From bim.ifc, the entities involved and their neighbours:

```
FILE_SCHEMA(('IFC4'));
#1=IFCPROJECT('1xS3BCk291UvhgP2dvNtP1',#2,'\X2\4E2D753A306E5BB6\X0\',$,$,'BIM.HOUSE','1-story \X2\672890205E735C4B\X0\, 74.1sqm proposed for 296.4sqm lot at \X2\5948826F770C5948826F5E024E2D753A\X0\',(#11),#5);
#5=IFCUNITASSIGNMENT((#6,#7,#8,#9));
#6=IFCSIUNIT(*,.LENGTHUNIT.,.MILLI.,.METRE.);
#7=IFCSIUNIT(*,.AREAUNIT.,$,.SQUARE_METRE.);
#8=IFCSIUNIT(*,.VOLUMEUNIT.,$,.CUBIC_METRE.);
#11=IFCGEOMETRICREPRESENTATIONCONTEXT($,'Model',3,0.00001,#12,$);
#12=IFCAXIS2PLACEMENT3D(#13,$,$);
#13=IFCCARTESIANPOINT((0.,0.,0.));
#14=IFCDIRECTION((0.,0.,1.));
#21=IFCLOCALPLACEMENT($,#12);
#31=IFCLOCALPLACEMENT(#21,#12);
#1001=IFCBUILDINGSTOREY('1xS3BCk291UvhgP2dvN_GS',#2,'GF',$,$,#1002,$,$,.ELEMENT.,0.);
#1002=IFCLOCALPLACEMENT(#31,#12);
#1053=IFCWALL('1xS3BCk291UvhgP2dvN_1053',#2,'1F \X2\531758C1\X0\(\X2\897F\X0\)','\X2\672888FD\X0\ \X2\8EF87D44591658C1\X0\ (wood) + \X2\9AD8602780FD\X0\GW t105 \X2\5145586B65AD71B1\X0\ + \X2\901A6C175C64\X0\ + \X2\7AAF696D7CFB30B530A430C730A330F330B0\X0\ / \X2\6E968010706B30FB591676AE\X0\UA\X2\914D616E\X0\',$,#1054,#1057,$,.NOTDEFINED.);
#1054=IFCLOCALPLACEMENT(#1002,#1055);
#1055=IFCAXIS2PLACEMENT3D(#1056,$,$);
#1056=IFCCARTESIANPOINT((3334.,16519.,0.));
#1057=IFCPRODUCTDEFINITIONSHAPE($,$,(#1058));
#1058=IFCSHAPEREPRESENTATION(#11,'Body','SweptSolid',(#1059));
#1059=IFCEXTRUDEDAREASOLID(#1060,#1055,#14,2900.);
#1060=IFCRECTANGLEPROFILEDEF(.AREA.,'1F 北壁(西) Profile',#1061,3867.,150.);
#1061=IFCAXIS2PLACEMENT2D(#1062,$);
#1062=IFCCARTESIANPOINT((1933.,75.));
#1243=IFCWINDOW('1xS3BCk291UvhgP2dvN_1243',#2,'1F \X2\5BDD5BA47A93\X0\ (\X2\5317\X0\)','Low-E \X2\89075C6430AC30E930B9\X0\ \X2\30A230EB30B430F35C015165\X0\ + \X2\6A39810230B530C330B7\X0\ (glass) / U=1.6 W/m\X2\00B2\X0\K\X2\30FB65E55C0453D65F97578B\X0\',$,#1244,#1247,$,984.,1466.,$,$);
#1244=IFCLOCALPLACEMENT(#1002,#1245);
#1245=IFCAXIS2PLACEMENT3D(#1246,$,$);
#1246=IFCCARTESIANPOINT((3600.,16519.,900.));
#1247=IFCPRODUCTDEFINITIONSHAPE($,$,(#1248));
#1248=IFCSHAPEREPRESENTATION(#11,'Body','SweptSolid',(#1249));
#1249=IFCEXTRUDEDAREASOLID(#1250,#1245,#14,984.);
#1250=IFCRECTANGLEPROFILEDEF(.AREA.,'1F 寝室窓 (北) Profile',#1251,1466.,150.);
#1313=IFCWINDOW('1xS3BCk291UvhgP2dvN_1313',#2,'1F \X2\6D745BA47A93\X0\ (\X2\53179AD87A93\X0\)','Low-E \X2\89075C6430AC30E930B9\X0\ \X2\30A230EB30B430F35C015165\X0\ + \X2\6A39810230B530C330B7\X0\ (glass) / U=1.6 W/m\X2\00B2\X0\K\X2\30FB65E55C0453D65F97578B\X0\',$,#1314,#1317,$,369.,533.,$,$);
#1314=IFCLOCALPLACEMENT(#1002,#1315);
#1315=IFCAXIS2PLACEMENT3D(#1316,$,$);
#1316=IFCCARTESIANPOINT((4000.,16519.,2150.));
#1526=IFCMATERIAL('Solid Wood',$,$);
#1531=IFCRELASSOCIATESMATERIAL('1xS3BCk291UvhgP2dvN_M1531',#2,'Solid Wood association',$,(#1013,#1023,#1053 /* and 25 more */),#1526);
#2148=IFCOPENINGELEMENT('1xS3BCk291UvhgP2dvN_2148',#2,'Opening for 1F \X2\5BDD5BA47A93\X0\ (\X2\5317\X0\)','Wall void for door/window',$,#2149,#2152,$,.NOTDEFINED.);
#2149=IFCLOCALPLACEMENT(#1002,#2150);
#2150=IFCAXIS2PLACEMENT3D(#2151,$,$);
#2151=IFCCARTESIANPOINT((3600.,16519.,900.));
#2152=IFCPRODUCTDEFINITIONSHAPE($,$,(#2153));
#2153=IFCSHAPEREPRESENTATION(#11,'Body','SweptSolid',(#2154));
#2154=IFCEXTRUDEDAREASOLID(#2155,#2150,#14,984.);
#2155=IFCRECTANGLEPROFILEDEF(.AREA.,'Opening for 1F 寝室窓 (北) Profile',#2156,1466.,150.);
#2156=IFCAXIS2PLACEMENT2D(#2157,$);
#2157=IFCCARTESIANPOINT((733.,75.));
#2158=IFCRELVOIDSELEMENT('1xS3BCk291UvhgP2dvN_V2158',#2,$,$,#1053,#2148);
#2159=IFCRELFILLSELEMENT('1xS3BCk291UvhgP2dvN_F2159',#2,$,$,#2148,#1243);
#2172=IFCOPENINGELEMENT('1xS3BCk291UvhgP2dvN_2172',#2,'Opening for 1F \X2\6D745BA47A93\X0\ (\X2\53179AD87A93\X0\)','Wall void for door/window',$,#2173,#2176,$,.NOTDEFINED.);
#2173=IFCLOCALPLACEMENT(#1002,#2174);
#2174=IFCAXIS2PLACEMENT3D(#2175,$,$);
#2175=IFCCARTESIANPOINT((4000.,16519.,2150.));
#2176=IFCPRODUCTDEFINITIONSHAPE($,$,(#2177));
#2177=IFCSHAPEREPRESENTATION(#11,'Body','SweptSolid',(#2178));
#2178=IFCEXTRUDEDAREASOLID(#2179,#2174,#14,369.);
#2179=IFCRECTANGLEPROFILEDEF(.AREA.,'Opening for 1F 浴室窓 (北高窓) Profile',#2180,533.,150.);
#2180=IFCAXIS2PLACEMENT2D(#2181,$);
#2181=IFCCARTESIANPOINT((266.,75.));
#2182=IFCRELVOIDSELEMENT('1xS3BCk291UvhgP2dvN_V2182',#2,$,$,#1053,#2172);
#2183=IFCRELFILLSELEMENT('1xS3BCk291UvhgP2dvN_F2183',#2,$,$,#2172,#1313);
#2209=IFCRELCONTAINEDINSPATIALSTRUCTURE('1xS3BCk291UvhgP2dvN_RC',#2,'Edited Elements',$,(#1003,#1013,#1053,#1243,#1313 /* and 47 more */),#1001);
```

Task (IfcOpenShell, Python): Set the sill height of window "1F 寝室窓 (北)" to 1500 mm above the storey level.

```python
import numpy as np
import ifcopenshell
import ifcopenshell.api.geometry
import ifcopenshell.geom
import ifcopenshell.util.element
import ifcopenshell.util.placement
import ifcopenshell.util.shape
import ifcopenshell.util.unit

model = ifcopenshell.open("bim.ifc")
unit_scale = ifcopenshell.util.unit.calculate_unit_scale(model)

window = model.by_id(1243)
opening = window.FillsVoids[0].RelatingOpeningElement
storey = ifcopenshell.util.element.get_container(window, ifc_class="IfcBuildingStorey")
level = ifcopenshell.util.placement.get_local_placement(storey.ObjectPlacement)[2, 3]

# The opening's origin need not be at the sill, so measure its lowest point.
shape = ifcopenshell.geom.create_shape(ifcopenshell.geom.settings(), opening)
bottom = ifcopenshell.util.shape.get_shape_bottom_elevation(shape, shape.geometry) / unit_scale
dz = level + 1500.0 - bottom

shift = np.array([0.0, 0.0, dz])
# The window is not placed relative to its opening, so move both.
for product in (opening, window):
    matrix = ifcopenshell.util.placement.get_local_placement(product.ObjectPlacement)
    matrix[:3, 3] += shift
    ifcopenshell.api.geometry.edit_object_placement(model, product=product, matrix=matrix, is_si=False)

print(f"moved by {dz * unit_scale:+.3f} m")

model.write("bim_updated.ifc")
```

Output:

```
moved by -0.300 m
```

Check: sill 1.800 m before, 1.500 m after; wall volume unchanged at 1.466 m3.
